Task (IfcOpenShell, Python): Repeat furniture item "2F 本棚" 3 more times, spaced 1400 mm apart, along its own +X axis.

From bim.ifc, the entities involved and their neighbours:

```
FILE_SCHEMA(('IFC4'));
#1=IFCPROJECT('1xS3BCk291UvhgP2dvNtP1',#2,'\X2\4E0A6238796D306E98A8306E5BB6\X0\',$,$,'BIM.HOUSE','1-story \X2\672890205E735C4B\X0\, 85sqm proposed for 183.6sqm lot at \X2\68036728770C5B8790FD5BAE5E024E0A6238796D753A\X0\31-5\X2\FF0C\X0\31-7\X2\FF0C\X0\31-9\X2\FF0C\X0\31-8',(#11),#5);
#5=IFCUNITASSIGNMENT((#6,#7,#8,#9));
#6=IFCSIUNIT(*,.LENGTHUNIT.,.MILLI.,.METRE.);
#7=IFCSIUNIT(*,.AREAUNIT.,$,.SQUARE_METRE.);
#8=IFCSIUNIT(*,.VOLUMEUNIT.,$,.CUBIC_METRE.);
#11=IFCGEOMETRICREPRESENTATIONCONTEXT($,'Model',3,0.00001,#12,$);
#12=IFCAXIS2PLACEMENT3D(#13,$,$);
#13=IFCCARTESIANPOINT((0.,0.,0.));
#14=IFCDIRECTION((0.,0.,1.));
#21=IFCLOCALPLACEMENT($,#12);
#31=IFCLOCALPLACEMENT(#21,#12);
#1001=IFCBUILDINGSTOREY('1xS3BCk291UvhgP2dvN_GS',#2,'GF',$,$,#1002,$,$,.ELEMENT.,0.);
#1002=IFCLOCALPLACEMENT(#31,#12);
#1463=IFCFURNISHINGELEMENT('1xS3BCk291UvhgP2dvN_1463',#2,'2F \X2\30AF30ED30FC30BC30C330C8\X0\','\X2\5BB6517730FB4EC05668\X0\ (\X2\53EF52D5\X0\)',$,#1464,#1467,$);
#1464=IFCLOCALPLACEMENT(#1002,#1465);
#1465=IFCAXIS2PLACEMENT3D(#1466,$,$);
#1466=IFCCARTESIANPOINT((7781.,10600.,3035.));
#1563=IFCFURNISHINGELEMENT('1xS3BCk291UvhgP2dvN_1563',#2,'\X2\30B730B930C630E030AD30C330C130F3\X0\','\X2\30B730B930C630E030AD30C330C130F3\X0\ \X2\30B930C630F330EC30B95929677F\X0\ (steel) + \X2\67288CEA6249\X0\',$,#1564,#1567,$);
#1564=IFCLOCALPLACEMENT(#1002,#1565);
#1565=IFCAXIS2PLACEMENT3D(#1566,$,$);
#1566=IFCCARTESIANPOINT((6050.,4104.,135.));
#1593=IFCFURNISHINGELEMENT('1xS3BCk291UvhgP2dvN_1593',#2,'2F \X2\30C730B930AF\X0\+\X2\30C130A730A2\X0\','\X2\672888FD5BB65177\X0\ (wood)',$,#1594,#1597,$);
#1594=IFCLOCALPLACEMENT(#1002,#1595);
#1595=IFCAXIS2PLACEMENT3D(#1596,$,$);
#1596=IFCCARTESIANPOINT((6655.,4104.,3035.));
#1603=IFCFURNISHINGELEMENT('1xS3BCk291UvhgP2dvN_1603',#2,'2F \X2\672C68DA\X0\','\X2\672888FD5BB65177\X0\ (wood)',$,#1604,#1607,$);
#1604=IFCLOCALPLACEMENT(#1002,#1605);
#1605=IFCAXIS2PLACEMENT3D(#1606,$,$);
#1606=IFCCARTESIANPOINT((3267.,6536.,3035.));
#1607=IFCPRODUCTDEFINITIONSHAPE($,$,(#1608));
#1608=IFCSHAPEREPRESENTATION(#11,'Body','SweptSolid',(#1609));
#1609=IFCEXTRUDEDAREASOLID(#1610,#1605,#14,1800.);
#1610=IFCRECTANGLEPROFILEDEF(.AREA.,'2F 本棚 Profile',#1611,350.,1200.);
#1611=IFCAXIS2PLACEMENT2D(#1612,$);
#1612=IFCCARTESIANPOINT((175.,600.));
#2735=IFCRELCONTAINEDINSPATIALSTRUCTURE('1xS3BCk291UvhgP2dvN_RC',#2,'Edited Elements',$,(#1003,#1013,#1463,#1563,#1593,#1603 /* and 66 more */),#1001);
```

```python
import ifcopenshell
import ifcopenshell.api.geometry
import ifcopenshell.api.root
import ifcopenshell.util.element
import ifcopenshell.util.placement
import ifcopenshell.util.unit

model = ifcopenshell.open("bim.ifc")
unit_scale = ifcopenshell.util.unit.calculate_unit_scale(model)


def reuse_history(source, copy):
    """copy_class also copies each property set's owner history, people and application; keep the originals."""
    for rel in copy.IsDefinedBy:
        if rel.is_a("IfcRelDefinesByProperties") and (history := rel.RelatingPropertyDefinition.OwnerHistory):
            rel.RelatingPropertyDefinition.OwnerHistory = source.OwnerHistory
            ifcopenshell.util.element.remove_deep2(model, history)


source = model.by_guid("1xS3BCk291UvhgP2dvN_1603")
base = ifcopenshell.util.placement.get_local_placement(source.ObjectPlacement)
step = base[:3, 0] * 1.4 / unit_scale

for i in range(1, 4):
    copy = ifcopenshell.api.root.copy_class(model, product=source)
    copy.Representation = ifcopenshell.util.element.copy_deep(
        model, source.Representation, exclude=["IfcGeometricRepresentationContext", "IfcRepresentationMap"]
    )
    reuse_history(source, copy)
    matrix = base.copy()
    matrix[:3, 3] += i * step
    print("added at", matrix[:3, 3].round(3) + 0.0)
    ifcopenshell.api.geometry.edit_object_placement(model, product=copy, matrix=matrix, is_si=False)

model.write("bim_edited.ifc")
```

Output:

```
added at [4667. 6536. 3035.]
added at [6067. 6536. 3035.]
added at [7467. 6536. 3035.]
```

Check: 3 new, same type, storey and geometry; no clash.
